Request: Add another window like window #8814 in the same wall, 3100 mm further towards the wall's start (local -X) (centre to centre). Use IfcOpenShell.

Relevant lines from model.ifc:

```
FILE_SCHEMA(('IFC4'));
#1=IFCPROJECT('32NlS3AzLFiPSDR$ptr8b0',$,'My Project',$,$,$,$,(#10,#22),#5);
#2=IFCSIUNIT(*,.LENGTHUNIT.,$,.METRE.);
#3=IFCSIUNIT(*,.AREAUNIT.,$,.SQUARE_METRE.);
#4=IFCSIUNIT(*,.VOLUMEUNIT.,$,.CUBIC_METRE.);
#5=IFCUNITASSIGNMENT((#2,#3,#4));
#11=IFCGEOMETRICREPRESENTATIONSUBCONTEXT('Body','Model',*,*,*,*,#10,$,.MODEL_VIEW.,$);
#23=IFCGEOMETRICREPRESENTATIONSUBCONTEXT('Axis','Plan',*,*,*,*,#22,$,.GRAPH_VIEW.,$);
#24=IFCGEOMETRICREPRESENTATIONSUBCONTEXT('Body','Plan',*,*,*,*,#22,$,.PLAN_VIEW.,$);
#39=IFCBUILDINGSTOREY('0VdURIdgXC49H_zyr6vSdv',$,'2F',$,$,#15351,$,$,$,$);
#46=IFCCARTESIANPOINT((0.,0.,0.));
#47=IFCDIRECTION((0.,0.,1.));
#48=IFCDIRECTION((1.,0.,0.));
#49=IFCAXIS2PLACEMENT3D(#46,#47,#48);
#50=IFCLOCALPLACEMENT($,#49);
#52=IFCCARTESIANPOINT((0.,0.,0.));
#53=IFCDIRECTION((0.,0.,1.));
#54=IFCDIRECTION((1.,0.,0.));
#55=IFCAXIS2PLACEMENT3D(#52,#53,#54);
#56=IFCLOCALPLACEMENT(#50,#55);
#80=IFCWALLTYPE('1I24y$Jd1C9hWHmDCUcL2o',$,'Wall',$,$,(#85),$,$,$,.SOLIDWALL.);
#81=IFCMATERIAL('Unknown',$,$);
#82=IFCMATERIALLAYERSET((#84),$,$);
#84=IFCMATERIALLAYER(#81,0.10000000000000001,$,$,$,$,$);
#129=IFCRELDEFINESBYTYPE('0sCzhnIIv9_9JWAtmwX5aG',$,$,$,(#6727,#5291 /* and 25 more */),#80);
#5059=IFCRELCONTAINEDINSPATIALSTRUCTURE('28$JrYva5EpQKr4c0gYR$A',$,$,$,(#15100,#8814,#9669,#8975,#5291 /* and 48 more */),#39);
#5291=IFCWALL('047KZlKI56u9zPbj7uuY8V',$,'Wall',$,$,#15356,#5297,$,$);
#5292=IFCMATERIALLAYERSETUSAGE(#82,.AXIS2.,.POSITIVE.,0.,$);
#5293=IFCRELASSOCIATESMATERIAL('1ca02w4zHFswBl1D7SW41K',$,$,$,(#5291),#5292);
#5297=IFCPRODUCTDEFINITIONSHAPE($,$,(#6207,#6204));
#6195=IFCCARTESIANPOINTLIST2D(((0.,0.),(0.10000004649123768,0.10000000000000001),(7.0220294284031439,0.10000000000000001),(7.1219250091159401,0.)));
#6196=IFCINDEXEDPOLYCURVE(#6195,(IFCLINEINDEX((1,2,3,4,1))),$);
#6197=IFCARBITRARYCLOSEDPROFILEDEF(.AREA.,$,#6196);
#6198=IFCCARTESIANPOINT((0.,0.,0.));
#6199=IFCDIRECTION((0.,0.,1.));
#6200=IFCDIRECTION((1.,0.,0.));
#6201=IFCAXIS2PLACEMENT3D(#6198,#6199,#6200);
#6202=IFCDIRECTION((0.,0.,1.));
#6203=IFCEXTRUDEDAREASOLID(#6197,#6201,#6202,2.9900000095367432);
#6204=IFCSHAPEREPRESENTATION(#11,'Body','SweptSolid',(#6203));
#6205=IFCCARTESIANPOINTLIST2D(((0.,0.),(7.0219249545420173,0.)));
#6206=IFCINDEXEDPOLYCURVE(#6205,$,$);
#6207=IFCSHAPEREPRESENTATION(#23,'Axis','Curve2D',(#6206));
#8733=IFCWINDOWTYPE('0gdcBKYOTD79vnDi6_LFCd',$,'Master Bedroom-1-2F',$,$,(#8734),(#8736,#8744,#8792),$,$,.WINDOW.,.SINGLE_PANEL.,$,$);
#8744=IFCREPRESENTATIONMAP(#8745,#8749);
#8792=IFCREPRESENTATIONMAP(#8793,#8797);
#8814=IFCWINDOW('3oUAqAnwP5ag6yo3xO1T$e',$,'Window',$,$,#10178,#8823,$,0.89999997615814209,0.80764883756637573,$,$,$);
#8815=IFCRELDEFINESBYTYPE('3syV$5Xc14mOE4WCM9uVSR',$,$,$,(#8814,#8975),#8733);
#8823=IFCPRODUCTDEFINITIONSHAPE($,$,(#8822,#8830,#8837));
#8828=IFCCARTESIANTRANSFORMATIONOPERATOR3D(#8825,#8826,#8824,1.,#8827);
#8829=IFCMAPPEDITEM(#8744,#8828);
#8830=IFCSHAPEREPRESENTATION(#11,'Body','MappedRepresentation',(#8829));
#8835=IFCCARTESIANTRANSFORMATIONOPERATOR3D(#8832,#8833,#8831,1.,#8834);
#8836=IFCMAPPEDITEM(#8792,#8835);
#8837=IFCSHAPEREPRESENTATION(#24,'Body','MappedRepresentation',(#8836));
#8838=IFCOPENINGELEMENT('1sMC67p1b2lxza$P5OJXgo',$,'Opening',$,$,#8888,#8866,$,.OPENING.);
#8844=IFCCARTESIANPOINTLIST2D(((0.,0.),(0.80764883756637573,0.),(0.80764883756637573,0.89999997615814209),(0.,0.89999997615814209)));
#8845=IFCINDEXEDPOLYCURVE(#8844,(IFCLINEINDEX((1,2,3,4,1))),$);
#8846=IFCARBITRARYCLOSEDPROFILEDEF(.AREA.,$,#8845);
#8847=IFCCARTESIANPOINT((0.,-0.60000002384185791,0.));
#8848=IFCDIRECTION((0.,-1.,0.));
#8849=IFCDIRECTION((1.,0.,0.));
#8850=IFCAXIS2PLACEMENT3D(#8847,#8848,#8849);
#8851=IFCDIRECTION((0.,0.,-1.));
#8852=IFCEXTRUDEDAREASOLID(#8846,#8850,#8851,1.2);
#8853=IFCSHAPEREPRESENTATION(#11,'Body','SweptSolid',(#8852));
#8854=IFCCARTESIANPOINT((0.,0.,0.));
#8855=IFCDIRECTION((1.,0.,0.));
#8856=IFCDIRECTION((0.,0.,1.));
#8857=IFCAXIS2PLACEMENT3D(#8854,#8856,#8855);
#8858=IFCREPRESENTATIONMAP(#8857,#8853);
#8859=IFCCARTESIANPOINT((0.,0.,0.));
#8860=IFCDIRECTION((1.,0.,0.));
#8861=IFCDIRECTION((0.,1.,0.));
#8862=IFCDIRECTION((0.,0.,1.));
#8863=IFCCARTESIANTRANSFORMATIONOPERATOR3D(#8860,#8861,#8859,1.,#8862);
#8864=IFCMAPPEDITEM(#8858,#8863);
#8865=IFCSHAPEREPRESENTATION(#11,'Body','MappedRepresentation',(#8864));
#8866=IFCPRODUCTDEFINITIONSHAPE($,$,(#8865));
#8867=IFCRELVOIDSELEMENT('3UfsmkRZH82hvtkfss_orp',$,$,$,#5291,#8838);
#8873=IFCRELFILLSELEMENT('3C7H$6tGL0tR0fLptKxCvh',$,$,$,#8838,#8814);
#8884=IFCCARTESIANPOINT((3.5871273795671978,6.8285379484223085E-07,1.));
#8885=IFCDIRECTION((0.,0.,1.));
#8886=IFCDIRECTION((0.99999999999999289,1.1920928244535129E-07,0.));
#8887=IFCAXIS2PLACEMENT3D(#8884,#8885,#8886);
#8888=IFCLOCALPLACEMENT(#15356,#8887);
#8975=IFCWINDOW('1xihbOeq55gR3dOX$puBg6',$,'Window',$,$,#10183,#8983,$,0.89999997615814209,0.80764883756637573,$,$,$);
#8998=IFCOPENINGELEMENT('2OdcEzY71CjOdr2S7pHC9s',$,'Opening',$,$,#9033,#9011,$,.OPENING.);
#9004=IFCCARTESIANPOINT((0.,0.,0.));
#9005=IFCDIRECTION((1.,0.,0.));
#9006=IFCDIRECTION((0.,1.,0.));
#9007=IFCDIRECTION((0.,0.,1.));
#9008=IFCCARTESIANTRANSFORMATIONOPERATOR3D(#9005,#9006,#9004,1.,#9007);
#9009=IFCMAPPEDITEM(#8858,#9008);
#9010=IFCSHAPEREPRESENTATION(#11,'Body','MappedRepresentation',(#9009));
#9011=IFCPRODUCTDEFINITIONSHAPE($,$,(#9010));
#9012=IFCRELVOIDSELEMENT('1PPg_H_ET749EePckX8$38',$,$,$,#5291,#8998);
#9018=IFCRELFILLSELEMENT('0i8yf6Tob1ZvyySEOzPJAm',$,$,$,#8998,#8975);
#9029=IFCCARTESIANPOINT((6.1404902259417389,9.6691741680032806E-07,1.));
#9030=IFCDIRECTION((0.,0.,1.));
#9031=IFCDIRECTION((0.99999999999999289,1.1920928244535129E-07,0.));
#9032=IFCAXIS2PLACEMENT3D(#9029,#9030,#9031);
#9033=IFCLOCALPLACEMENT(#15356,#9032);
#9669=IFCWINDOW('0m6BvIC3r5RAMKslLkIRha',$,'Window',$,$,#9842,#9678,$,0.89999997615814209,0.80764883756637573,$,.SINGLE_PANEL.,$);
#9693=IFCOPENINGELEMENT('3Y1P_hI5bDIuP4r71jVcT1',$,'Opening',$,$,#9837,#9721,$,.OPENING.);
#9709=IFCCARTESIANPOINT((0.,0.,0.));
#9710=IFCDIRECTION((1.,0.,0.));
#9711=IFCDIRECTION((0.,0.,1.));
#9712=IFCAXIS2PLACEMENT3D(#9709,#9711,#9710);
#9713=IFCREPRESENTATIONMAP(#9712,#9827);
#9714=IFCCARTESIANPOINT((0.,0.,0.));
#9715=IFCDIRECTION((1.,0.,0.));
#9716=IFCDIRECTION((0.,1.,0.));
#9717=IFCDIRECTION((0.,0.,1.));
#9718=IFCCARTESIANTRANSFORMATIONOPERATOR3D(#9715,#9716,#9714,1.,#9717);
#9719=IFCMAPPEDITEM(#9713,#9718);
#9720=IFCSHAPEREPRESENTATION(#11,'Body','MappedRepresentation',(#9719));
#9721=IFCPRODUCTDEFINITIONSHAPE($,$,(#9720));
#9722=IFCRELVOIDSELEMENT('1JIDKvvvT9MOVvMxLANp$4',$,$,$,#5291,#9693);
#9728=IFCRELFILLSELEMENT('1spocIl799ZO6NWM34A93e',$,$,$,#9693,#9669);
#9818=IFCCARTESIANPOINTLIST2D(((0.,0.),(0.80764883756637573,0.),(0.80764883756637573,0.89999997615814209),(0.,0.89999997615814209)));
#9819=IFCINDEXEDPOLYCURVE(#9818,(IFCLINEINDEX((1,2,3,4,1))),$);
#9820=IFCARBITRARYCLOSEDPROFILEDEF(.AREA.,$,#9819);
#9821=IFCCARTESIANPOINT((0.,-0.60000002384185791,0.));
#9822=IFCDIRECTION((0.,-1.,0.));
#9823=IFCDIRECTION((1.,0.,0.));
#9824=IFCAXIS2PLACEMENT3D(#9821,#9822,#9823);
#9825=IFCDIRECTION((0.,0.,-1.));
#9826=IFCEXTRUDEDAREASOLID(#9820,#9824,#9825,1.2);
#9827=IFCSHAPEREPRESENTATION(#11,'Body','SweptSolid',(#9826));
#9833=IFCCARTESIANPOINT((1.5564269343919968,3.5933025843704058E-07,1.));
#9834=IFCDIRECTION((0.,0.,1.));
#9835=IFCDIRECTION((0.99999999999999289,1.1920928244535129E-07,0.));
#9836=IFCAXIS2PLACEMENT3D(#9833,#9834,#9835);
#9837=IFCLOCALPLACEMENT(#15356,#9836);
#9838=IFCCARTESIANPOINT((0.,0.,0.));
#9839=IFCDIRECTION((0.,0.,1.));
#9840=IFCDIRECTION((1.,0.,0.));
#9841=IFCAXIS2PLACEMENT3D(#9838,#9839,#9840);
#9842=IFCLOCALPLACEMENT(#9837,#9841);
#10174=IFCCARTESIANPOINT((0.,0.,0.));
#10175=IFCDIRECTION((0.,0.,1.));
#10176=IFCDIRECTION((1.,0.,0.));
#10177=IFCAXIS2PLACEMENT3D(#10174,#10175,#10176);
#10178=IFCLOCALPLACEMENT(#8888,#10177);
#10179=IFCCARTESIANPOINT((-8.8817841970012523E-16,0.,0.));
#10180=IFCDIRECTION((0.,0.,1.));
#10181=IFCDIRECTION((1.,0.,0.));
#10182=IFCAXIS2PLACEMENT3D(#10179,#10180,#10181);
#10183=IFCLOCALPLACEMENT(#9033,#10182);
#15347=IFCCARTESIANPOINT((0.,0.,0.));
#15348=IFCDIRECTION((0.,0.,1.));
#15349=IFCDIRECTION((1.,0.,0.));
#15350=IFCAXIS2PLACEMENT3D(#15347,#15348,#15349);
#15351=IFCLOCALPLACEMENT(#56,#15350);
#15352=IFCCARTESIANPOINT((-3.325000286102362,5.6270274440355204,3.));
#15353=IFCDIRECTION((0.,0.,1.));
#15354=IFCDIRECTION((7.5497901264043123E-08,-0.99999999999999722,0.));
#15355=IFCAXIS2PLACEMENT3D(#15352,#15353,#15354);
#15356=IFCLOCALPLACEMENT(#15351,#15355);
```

```python
import ifcopenshell
import ifcopenshell.api.feature
import ifcopenshell.api.geometry
import ifcopenshell.api.root
import ifcopenshell.geom
import ifcopenshell.util.element
import ifcopenshell.util.placement
import ifcopenshell.util.shape
import ifcopenshell.util.unit

model = ifcopenshell.open("model.ifc")
unit_scale = ifcopenshell.util.unit.calculate_unit_scale(model)
settings = ifcopenshell.geom.settings()


def volume(element):
    """Net volume in cubic metres, openings subtracted."""
    shape = ifcopenshell.geom.create_shape(settings, element)
    return ifcopenshell.util.shape.get_volume(shape.geometry)


window = model.by_guid("3oUAqAnwP5ag6yo3xO1T$e")
opening = window.FillsVoids[0].RelatingOpeningElement
wall = opening.VoidsElements[0].RelatingBuildingElement
before = volume(wall)
shift = ifcopenshell.util.placement.get_local_placement(wall.ObjectPlacement)[:3, 0] * -3.1 / unit_scale

# copy_class copies the void relationship, type, container and properties, but no geometry.
new_opening = ifcopenshell.api.root.copy_class(model, product=opening)
new_opening.Representation = ifcopenshell.util.element.copy_deep(
    model, opening.Representation, exclude=["IfcGeometricRepresentationContext", "IfcRepresentationMap"]
)
new_window = ifcopenshell.api.root.copy_class(model, product=window)
new_window.Representation = ifcopenshell.util.element.copy_deep(
    model, window.Representation, exclude=["IfcGeometricRepresentationContext", "IfcRepresentationMap"]
)
ifcopenshell.api.feature.add_filling(model, opening=new_opening, element=new_window)

for old, new in ((opening, new_opening), (window, new_window)):
    matrix = ifcopenshell.util.placement.get_local_placement(old.ObjectPlacement)
    matrix[:3, 3] += shift
    ifcopenshell.api.geometry.edit_object_placement(model, product=new, matrix=matrix, is_si=False)

after = volume(wall)

print(f"wall volume {before:.3f} -> {after:.3f} m3")

model.write("model_edited.ifc")
```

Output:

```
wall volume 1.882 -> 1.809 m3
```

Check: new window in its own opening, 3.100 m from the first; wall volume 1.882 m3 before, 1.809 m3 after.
